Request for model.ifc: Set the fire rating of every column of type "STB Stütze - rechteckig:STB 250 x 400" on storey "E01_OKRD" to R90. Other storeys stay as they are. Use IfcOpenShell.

First a look at what the model holds.

```python
import ifcopenshell
import ifcopenshell.util.element

model = ifcopenshell.open("model.ifc")
print(model.schema)
storey = next(s for s in model.by_type("IfcBuildingStorey") if s.Name == "E01_OKRD")
columns = [e for e in ifcopenshell.util.element.get_decomposition(storey) if e.is_a("IfcColumn")]
seen = {}
for e in columns:
    element_type = ifcopenshell.util.element.get_type(e)
    key = (element_type.Name if element_type != e and element_type else None, ifcopenshell.util.element.get_pset(e, "Pset_ColumnCommon", "FireRating"))
    seen[key] = seen.get(key, 0) + 1
for (name, value), count in sorted(seen.items(), key=str):
    print(count, "x", name, "|", value)
```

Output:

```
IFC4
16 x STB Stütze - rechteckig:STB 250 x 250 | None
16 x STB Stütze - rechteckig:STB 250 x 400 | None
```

```python
import ifcopenshell
import ifcopenshell.api.pset
import ifcopenshell.util.element

model = ifcopenshell.open("model.ifc")

storey = next(s for s in model.by_type("IfcBuildingStorey") if s.Name == "E01_OKRD")
columns = [e for e in ifcopenshell.util.element.get_decomposition(storey) if e.is_a("IfcColumn")]

count = 0
for e in columns:
    element_type = ifcopenshell.util.element.get_type(e)
    if element_type in (None, e) or element_type.Name != "STB Stütze - rechteckig:STB 250 x 400":
        continue
    # add_pset returns the element's existing set when there is one.
    pset = ifcopenshell.api.pset.add_pset(model, product=e, name="Pset_ColumnCommon")
    ifcopenshell.api.pset.edit_pset(model, pset=pset, properties={"FireRating": "R90"})
    count += 1

print(count, "columns updated")

model.write("model_edited.ifc")
```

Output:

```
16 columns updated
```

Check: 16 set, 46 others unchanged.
